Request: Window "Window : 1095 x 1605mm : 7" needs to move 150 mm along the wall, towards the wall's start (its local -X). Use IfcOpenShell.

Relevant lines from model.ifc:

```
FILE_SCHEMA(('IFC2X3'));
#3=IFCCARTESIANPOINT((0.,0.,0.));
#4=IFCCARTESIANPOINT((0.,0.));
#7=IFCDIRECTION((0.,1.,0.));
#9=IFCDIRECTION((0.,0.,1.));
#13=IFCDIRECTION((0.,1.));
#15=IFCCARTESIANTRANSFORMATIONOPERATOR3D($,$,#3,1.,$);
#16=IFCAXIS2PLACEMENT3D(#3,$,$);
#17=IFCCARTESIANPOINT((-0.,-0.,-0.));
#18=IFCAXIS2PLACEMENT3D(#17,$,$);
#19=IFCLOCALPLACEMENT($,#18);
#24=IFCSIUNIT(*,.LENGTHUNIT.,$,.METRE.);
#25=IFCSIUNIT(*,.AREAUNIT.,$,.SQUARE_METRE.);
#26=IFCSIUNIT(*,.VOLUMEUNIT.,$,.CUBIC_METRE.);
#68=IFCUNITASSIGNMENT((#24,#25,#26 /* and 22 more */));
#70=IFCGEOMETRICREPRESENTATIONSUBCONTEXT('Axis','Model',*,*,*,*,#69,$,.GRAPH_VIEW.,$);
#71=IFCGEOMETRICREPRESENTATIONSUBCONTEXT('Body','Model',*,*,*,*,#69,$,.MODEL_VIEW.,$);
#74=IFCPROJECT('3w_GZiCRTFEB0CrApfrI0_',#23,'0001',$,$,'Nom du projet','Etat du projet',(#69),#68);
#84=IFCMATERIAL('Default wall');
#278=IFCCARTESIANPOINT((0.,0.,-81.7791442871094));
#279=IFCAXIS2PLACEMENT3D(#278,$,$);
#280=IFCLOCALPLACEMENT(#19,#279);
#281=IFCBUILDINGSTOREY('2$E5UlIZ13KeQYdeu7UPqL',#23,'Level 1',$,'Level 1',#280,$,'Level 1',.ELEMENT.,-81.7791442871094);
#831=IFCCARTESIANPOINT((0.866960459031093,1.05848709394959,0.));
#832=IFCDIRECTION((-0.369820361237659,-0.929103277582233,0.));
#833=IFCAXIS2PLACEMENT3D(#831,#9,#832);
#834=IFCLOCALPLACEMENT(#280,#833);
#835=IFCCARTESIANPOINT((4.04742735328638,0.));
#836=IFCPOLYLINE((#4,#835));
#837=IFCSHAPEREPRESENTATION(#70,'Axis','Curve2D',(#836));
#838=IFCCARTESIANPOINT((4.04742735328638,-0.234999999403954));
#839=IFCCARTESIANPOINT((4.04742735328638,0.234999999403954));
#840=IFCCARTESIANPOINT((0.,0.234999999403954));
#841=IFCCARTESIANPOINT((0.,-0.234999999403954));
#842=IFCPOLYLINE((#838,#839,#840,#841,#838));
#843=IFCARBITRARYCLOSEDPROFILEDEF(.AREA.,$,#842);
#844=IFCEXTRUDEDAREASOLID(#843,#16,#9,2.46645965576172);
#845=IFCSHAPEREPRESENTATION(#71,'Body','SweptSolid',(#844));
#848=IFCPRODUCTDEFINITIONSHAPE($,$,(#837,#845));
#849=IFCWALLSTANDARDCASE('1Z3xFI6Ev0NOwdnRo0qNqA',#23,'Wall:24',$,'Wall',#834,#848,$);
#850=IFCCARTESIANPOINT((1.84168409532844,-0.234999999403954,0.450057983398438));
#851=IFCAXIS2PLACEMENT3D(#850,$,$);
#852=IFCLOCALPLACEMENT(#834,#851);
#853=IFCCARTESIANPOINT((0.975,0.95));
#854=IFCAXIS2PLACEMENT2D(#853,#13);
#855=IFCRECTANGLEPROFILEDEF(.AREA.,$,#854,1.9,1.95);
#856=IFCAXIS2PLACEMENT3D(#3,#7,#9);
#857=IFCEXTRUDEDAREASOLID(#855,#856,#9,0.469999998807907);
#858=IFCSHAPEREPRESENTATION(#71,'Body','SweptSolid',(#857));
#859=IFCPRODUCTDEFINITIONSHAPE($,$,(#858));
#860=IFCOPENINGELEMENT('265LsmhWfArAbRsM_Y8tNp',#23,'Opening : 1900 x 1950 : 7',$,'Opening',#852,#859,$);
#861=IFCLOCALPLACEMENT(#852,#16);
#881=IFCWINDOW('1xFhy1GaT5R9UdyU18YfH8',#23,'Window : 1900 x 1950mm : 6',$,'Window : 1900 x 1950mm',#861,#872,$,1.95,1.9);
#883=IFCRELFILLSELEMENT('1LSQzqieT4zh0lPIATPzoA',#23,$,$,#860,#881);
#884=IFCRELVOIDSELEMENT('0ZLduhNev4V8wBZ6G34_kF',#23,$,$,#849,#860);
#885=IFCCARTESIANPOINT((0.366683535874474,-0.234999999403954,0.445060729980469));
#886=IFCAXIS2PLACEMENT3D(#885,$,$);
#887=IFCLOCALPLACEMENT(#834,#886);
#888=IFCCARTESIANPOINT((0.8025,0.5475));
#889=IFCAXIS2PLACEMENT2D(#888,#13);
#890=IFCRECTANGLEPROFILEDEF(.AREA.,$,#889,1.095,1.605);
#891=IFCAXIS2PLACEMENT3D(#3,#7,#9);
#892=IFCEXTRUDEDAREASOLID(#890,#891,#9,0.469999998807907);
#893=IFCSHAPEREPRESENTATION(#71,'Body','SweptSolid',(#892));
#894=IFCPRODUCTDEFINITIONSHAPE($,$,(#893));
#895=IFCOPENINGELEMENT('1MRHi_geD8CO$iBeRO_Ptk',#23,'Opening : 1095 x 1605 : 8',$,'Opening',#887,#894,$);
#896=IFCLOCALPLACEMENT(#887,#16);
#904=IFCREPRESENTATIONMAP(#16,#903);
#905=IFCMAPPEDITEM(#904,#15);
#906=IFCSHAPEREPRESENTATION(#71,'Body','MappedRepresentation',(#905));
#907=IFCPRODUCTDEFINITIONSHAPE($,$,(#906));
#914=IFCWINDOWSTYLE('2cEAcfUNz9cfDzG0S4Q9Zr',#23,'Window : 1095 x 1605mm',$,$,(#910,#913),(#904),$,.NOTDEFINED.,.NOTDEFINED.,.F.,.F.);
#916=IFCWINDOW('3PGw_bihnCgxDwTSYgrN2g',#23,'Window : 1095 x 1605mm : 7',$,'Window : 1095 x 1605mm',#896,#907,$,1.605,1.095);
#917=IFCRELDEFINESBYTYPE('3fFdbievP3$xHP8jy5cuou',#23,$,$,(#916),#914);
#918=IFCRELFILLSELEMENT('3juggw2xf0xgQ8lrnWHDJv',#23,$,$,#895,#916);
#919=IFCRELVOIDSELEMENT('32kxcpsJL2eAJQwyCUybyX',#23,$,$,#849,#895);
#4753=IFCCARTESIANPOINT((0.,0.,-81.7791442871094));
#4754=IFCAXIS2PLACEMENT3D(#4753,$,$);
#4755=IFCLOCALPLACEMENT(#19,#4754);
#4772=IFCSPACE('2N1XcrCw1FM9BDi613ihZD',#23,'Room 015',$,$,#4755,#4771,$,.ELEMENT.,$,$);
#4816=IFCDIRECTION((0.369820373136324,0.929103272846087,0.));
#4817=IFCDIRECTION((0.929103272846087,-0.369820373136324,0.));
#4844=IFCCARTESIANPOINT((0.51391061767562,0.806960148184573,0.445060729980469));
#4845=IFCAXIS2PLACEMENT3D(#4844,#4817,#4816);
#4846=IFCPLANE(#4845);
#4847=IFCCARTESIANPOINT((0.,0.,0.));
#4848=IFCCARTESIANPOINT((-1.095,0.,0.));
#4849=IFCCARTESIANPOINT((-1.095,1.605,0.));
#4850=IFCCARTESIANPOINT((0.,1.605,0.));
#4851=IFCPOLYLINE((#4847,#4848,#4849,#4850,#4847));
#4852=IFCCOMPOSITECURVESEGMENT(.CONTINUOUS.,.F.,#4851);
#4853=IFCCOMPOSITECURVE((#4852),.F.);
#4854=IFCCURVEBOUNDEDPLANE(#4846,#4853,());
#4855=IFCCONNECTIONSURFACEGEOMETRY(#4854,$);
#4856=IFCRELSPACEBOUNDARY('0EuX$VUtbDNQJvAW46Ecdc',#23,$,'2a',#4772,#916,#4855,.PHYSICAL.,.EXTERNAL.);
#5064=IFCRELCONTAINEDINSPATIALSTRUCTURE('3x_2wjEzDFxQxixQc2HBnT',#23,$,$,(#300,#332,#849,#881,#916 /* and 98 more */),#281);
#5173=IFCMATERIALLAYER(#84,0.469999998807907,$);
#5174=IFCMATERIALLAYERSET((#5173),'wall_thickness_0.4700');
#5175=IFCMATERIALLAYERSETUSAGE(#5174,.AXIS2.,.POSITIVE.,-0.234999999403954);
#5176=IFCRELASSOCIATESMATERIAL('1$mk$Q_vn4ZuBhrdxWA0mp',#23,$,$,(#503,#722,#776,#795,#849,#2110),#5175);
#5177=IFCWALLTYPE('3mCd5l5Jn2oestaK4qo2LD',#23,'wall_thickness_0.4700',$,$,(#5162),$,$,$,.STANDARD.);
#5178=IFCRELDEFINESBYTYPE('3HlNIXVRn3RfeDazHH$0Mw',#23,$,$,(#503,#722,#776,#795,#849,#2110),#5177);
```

```python
import numpy as np
import ifcopenshell
import ifcopenshell.api.geometry
import ifcopenshell.util.placement
import ifcopenshell.util.unit

model = ifcopenshell.open("model.ifc")
unit_scale = ifcopenshell.util.unit.calculate_unit_scale(model)

window = model.by_id(916)
opening = window.FillsVoids[0].RelatingOpeningElement
wall = opening.VoidsElements[0].RelatingBuildingElement

wall_matrix = ifcopenshell.util.placement.get_local_placement(wall.ObjectPlacement)
shift = wall_matrix[:3, 0] * -0.15 / unit_scale
before = ifcopenshell.util.placement.get_local_placement(window.ObjectPlacement)[:3, 3].copy()

# The window is placed relative to its opening, so it follows when the opening moves.
matrix = ifcopenshell.util.placement.get_local_placement(opening.ObjectPlacement)
matrix[:3, 3] += shift
ifcopenshell.api.geometry.edit_object_placement(
    model, product=opening, matrix=matrix, is_si=False, should_transform_children=True
)

# Space boundary surfaces are stored in each space's coordinates; move them too.
for rel in window.ProvidesBoundaries:
    if not rel.ConnectionGeometry:
        continue
    surface = rel.ConnectionGeometry.SurfaceOnRelatingElement.BasisSurface
    space_matrix = ifcopenshell.util.placement.get_local_placement(rel.RelatingSpace.ObjectPlacement)
    point = np.array(surface.Position.Location.Coordinates) + space_matrix[:3, :3].T @ shift
    surface.Position = model.createIfcAxis2Placement3D(
        model.createIfcCartesianPoint(point.tolist()), surface.Position.Axis, surface.Position.RefDirection
    )

after = ifcopenshell.util.placement.get_local_placement(window.ObjectPlacement)[:3, 3]
print("window moved by", (after - before).round(3) + 0.0)

model.write("model_updated.ifc")
```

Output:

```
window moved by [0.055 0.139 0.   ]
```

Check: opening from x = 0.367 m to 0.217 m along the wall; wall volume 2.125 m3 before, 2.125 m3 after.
